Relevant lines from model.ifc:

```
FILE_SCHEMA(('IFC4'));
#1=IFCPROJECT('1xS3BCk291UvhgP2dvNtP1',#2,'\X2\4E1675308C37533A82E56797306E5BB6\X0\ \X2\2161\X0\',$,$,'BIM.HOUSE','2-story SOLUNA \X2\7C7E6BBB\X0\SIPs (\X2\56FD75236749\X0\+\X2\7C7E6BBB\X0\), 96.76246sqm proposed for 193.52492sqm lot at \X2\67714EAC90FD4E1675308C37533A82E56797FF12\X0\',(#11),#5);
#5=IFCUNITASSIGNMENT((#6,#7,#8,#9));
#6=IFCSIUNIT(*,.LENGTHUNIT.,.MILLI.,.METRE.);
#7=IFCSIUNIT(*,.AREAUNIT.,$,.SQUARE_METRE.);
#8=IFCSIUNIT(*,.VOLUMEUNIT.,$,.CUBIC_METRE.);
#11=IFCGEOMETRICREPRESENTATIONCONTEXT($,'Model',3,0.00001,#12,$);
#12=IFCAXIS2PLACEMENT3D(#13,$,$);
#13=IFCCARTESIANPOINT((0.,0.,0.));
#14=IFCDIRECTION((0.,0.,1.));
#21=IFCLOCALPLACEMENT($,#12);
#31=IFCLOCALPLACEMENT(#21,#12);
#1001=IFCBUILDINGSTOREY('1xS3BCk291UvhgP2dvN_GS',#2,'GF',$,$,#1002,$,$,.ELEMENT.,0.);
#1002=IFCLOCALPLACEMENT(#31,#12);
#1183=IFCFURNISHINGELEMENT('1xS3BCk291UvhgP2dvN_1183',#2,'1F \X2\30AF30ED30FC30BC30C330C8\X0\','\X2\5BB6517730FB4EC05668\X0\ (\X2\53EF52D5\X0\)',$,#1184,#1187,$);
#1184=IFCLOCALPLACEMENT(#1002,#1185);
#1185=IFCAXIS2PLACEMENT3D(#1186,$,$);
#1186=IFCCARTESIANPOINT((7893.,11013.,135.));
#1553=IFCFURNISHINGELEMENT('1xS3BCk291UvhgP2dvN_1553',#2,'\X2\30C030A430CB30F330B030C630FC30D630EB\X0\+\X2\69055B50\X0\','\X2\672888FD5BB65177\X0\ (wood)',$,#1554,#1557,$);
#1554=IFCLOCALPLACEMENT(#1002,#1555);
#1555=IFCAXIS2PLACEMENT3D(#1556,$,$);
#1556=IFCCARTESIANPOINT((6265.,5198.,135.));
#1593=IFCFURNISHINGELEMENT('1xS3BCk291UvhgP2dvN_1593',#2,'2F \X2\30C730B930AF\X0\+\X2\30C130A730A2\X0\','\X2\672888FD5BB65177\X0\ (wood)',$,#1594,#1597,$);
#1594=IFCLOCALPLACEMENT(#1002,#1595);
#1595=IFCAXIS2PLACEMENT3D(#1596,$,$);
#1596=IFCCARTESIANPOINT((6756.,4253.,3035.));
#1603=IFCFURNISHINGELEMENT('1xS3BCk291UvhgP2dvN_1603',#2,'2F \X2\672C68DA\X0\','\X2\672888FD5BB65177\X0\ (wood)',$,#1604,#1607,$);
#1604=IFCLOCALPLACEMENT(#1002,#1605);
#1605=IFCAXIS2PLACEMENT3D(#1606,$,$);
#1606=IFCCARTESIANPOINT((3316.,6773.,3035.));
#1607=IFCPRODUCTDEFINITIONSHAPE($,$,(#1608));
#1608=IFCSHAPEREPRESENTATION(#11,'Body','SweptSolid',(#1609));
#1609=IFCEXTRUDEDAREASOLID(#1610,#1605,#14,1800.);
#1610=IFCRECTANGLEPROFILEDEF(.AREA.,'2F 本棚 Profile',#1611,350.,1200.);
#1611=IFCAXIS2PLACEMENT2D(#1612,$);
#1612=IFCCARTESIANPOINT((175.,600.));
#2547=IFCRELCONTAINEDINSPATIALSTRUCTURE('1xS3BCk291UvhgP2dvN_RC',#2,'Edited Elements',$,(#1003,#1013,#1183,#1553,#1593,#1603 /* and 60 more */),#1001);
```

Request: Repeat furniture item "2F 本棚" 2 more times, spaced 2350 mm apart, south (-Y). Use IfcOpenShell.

```python
import numpy as np
import ifcopenshell
import ifcopenshell.api.geometry
import ifcopenshell.api.root
import ifcopenshell.util.element
import ifcopenshell.util.placement
import ifcopenshell.util.unit

model = ifcopenshell.open("model.ifc")
unit_scale = ifcopenshell.util.unit.calculate_unit_scale(model)


def reuse_history(source, copy):
    """copy_class also copies each property set's owner history, people and application; keep the originals."""
    for rel in copy.IsDefinedBy:
        if rel.is_a("IfcRelDefinesByProperties") and (history := rel.RelatingPropertyDefinition.OwnerHistory):
            rel.RelatingPropertyDefinition.OwnerHistory = source.OwnerHistory
            ifcopenshell.util.element.remove_deep2(model, history)


source = model.by_guid("1xS3BCk291UvhgP2dvN_1603")
base = ifcopenshell.util.placement.get_local_placement(source.ObjectPlacement)
step = np.array([0.0, -1.0, 0.0]) * 2.35 / unit_scale

for i in range(1, 3):
    copy = ifcopenshell.api.root.copy_class(model, product=source)
    copy.Representation = ifcopenshell.util.element.copy_deep(
        model, source.Representation, exclude=["IfcGeometricRepresentationContext", "IfcRepresentationMap"]
    )
    reuse_history(source, copy)
    matrix = base.copy()
    matrix[:3, 3] += i * step
    print("added at", matrix[:3, 3].round(3) + 0.0)
    ifcopenshell.api.geometry.edit_object_placement(model, product=copy, matrix=matrix, is_si=False)

model.write("model_updated.ifc")
```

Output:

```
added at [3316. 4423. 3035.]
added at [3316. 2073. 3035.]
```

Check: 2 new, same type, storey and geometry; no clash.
